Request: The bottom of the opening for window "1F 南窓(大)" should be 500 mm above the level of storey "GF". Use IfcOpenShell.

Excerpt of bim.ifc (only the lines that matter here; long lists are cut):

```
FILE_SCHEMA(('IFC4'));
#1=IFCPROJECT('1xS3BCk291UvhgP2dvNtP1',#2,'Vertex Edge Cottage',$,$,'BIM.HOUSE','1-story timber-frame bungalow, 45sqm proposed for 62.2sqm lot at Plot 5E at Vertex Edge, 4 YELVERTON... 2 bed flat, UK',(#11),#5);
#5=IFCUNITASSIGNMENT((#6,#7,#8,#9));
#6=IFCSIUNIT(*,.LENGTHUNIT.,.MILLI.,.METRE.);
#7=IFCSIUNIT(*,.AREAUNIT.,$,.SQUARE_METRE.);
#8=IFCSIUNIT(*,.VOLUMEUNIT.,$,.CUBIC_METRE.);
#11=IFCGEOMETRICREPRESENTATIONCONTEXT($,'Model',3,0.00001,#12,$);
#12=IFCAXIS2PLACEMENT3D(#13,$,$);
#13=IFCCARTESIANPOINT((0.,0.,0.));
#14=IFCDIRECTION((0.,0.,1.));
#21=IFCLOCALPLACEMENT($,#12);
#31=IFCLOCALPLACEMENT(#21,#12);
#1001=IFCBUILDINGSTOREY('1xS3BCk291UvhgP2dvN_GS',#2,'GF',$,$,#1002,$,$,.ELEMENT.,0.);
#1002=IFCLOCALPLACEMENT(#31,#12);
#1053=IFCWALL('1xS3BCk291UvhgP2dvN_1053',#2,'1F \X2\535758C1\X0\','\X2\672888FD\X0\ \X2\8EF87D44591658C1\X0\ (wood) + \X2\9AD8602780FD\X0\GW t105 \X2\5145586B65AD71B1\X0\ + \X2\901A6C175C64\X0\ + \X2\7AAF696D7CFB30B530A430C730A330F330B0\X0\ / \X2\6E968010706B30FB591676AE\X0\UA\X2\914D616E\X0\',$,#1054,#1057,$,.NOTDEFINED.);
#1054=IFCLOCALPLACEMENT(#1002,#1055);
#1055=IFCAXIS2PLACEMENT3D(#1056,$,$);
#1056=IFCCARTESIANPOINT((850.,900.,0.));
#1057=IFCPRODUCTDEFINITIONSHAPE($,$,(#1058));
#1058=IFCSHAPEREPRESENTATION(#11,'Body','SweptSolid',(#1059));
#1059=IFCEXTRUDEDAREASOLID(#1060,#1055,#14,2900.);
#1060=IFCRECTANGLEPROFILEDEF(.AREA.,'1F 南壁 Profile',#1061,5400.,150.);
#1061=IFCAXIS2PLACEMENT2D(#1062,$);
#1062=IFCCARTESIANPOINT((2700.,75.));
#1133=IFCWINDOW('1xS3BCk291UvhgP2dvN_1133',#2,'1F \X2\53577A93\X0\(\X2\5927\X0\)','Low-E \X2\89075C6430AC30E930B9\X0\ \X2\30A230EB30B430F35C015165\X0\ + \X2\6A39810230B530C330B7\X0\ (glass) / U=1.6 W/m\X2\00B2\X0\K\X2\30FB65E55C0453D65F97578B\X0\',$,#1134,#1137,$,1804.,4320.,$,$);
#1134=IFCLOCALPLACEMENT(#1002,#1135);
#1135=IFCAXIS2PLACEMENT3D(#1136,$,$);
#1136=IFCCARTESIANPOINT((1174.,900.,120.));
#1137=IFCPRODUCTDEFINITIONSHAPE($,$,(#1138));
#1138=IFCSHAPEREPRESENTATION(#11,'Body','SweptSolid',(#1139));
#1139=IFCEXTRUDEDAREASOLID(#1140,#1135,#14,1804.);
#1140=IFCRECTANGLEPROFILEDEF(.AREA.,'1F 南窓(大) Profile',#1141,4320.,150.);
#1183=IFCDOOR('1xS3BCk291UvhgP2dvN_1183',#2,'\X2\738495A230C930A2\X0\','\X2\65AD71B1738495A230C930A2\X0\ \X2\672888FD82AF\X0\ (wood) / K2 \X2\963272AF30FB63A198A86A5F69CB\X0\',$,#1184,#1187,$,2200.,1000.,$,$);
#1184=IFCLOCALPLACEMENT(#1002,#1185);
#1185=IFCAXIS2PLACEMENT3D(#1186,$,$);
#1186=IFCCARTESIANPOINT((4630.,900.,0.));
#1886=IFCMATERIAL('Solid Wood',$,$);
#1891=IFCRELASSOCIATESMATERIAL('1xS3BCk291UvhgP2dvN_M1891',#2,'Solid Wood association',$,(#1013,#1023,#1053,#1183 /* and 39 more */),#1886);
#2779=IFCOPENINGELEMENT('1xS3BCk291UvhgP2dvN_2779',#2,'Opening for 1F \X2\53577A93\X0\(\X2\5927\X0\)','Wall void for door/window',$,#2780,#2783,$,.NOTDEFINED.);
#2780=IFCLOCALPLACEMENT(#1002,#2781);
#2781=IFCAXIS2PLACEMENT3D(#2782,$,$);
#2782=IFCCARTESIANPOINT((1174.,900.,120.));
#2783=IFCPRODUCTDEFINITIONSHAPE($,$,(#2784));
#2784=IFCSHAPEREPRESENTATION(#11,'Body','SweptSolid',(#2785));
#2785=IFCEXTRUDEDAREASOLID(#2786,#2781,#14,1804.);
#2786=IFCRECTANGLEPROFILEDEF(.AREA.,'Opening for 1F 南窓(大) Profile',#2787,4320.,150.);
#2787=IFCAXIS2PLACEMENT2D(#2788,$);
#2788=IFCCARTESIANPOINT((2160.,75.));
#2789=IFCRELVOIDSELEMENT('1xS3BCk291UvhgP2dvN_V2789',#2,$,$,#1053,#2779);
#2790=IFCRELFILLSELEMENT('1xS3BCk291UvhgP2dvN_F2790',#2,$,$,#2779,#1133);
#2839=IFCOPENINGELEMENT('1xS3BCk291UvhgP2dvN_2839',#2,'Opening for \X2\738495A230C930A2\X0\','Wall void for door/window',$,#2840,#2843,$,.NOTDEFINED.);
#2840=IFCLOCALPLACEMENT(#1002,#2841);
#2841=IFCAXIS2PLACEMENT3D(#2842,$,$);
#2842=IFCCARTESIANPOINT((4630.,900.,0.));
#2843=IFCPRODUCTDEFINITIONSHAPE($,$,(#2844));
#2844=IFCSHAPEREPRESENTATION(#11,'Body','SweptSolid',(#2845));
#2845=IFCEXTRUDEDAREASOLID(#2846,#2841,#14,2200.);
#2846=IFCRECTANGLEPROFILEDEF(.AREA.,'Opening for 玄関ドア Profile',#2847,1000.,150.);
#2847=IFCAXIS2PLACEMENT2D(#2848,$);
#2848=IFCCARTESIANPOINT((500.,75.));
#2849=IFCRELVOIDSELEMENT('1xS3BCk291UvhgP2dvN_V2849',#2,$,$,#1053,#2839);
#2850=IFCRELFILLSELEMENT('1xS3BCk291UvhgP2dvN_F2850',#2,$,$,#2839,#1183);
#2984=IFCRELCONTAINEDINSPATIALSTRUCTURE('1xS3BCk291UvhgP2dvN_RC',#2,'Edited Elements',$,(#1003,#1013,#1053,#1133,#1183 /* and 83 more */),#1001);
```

```python
import numpy as np
import ifcopenshell
import ifcopenshell.api.geometry
import ifcopenshell.geom
import ifcopenshell.util.element
import ifcopenshell.util.placement
import ifcopenshell.util.shape
import ifcopenshell.util.unit

model = ifcopenshell.open("bim.ifc")
unit_scale = ifcopenshell.util.unit.calculate_unit_scale(model)

window = model.by_guid("1xS3BCk291UvhgP2dvN_1133")
opening = window.FillsVoids[0].RelatingOpeningElement
storey = ifcopenshell.util.element.get_container(window, ifc_class="IfcBuildingStorey")
level = ifcopenshell.util.placement.get_local_placement(storey.ObjectPlacement)[2, 3]

# The opening's origin need not be at the sill, so measure its lowest point.
shape = ifcopenshell.geom.create_shape(ifcopenshell.geom.settings(), opening)
bottom = ifcopenshell.util.shape.get_shape_bottom_elevation(shape, shape.geometry) / unit_scale
dz = level + 500.0 - bottom

shift = np.array([0.0, 0.0, dz])
# The window is not placed relative to its opening, so move both.
for product in (opening, window):
    matrix = ifcopenshell.util.placement.get_local_placement(product.ObjectPlacement)
    matrix[:3, 3] += shift
    ifcopenshell.api.geometry.edit_object_placement(model, product=product, matrix=matrix, is_si=False)

print(f"moved by {dz * unit_scale:+.3f} m")

model.write("bim_updated.ifc")
```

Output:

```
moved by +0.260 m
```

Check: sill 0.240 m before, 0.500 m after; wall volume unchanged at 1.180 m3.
